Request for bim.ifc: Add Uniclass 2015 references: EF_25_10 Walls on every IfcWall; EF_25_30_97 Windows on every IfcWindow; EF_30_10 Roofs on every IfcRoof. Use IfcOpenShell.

First a look at what the model holds.

```python
import ifcopenshell

model = ifcopenshell.open("bim.ifc")
print(model.schema)
print("classifications:", [c.Name for c in model.by_type("IfcClassification")])
for ifc_class in ("IfcDoor", "IfcRoof", "IfcStair", "IfcWall", "IfcWindow"):
    print(ifc_class, len(model.by_type(ifc_class)))
```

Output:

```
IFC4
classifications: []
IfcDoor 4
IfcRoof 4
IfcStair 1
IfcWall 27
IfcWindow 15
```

```python
import ifcopenshell
import ifcopenshell.api.classification

model = ifcopenshell.open("bim.ifc")

system = ifcopenshell.api.classification.add_classification(model, classification="Uniclass 2015")

codes = {
    "IfcWall": ("EF_25_10", "Walls"),
    "IfcWindow": ("EF_25_30_97", "Windows"),
    "IfcRoof": ("EF_30_10", "Roofs"),
}
for ifc_class, (code, name) in codes.items():
    products = model.by_type(ifc_class)
    ifcopenshell.api.classification.add_reference(
        model, products=products, classification=system, identification=code, name=name
    )
    print(code, len(products))

model.write("bim_v2.ifc")
```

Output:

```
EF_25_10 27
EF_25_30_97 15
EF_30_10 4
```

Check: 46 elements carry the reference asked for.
